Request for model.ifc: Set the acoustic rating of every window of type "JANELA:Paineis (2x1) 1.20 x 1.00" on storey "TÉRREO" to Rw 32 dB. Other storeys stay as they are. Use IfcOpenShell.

First a look at what the model holds.

```python
import ifcopenshell
import ifcopenshell.util.element

model = ifcopenshell.open("model.ifc")
print(model.schema)
storey = next(s for s in model.by_type("IfcBuildingStorey") if s.Name == "TÉRREO")
windows = [e for e in ifcopenshell.util.element.get_decomposition(storey) if e.is_a("IfcWindow")]
seen = {}
for e in windows:
    element_type = ifcopenshell.util.element.get_type(e)
    key = (element_type.Name if element_type != e and element_type else None, ifcopenshell.util.element.get_pset(e, "Pset_WindowCommon", "AcousticRating"))
    seen[key] = seen.get(key, 0) + 1
for (name, value), count in sorted(seen.items(), key=str):
    print(count, "x", name, "|", value)
```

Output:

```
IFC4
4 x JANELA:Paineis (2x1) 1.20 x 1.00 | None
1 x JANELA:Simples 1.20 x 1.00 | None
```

```python
import ifcopenshell
import ifcopenshell.api.pset
import ifcopenshell.util.element

model = ifcopenshell.open("model.ifc")

storey = next(s for s in model.by_type("IfcBuildingStorey") if s.Name == "TÉRREO")
windows = [e for e in ifcopenshell.util.element.get_decomposition(storey) if e.is_a("IfcWindow")]

count = 0
for e in windows:
    element_type = ifcopenshell.util.element.get_type(e)
    if element_type in (None, e) or element_type.Name != "JANELA:Paineis (2x1) 1.20 x 1.00":
        continue
    # add_pset returns the element's existing set when there is one.
    pset = ifcopenshell.api.pset.add_pset(model, product=e, name="Pset_WindowCommon")
    ifcopenshell.api.pset.edit_pset(model, pset=pset, properties={"AcousticRating": "Rw 32 dB"})
    count += 1

print(count, "windows updated")

model.write("model_updated.ifc")
```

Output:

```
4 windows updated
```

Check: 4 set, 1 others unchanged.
